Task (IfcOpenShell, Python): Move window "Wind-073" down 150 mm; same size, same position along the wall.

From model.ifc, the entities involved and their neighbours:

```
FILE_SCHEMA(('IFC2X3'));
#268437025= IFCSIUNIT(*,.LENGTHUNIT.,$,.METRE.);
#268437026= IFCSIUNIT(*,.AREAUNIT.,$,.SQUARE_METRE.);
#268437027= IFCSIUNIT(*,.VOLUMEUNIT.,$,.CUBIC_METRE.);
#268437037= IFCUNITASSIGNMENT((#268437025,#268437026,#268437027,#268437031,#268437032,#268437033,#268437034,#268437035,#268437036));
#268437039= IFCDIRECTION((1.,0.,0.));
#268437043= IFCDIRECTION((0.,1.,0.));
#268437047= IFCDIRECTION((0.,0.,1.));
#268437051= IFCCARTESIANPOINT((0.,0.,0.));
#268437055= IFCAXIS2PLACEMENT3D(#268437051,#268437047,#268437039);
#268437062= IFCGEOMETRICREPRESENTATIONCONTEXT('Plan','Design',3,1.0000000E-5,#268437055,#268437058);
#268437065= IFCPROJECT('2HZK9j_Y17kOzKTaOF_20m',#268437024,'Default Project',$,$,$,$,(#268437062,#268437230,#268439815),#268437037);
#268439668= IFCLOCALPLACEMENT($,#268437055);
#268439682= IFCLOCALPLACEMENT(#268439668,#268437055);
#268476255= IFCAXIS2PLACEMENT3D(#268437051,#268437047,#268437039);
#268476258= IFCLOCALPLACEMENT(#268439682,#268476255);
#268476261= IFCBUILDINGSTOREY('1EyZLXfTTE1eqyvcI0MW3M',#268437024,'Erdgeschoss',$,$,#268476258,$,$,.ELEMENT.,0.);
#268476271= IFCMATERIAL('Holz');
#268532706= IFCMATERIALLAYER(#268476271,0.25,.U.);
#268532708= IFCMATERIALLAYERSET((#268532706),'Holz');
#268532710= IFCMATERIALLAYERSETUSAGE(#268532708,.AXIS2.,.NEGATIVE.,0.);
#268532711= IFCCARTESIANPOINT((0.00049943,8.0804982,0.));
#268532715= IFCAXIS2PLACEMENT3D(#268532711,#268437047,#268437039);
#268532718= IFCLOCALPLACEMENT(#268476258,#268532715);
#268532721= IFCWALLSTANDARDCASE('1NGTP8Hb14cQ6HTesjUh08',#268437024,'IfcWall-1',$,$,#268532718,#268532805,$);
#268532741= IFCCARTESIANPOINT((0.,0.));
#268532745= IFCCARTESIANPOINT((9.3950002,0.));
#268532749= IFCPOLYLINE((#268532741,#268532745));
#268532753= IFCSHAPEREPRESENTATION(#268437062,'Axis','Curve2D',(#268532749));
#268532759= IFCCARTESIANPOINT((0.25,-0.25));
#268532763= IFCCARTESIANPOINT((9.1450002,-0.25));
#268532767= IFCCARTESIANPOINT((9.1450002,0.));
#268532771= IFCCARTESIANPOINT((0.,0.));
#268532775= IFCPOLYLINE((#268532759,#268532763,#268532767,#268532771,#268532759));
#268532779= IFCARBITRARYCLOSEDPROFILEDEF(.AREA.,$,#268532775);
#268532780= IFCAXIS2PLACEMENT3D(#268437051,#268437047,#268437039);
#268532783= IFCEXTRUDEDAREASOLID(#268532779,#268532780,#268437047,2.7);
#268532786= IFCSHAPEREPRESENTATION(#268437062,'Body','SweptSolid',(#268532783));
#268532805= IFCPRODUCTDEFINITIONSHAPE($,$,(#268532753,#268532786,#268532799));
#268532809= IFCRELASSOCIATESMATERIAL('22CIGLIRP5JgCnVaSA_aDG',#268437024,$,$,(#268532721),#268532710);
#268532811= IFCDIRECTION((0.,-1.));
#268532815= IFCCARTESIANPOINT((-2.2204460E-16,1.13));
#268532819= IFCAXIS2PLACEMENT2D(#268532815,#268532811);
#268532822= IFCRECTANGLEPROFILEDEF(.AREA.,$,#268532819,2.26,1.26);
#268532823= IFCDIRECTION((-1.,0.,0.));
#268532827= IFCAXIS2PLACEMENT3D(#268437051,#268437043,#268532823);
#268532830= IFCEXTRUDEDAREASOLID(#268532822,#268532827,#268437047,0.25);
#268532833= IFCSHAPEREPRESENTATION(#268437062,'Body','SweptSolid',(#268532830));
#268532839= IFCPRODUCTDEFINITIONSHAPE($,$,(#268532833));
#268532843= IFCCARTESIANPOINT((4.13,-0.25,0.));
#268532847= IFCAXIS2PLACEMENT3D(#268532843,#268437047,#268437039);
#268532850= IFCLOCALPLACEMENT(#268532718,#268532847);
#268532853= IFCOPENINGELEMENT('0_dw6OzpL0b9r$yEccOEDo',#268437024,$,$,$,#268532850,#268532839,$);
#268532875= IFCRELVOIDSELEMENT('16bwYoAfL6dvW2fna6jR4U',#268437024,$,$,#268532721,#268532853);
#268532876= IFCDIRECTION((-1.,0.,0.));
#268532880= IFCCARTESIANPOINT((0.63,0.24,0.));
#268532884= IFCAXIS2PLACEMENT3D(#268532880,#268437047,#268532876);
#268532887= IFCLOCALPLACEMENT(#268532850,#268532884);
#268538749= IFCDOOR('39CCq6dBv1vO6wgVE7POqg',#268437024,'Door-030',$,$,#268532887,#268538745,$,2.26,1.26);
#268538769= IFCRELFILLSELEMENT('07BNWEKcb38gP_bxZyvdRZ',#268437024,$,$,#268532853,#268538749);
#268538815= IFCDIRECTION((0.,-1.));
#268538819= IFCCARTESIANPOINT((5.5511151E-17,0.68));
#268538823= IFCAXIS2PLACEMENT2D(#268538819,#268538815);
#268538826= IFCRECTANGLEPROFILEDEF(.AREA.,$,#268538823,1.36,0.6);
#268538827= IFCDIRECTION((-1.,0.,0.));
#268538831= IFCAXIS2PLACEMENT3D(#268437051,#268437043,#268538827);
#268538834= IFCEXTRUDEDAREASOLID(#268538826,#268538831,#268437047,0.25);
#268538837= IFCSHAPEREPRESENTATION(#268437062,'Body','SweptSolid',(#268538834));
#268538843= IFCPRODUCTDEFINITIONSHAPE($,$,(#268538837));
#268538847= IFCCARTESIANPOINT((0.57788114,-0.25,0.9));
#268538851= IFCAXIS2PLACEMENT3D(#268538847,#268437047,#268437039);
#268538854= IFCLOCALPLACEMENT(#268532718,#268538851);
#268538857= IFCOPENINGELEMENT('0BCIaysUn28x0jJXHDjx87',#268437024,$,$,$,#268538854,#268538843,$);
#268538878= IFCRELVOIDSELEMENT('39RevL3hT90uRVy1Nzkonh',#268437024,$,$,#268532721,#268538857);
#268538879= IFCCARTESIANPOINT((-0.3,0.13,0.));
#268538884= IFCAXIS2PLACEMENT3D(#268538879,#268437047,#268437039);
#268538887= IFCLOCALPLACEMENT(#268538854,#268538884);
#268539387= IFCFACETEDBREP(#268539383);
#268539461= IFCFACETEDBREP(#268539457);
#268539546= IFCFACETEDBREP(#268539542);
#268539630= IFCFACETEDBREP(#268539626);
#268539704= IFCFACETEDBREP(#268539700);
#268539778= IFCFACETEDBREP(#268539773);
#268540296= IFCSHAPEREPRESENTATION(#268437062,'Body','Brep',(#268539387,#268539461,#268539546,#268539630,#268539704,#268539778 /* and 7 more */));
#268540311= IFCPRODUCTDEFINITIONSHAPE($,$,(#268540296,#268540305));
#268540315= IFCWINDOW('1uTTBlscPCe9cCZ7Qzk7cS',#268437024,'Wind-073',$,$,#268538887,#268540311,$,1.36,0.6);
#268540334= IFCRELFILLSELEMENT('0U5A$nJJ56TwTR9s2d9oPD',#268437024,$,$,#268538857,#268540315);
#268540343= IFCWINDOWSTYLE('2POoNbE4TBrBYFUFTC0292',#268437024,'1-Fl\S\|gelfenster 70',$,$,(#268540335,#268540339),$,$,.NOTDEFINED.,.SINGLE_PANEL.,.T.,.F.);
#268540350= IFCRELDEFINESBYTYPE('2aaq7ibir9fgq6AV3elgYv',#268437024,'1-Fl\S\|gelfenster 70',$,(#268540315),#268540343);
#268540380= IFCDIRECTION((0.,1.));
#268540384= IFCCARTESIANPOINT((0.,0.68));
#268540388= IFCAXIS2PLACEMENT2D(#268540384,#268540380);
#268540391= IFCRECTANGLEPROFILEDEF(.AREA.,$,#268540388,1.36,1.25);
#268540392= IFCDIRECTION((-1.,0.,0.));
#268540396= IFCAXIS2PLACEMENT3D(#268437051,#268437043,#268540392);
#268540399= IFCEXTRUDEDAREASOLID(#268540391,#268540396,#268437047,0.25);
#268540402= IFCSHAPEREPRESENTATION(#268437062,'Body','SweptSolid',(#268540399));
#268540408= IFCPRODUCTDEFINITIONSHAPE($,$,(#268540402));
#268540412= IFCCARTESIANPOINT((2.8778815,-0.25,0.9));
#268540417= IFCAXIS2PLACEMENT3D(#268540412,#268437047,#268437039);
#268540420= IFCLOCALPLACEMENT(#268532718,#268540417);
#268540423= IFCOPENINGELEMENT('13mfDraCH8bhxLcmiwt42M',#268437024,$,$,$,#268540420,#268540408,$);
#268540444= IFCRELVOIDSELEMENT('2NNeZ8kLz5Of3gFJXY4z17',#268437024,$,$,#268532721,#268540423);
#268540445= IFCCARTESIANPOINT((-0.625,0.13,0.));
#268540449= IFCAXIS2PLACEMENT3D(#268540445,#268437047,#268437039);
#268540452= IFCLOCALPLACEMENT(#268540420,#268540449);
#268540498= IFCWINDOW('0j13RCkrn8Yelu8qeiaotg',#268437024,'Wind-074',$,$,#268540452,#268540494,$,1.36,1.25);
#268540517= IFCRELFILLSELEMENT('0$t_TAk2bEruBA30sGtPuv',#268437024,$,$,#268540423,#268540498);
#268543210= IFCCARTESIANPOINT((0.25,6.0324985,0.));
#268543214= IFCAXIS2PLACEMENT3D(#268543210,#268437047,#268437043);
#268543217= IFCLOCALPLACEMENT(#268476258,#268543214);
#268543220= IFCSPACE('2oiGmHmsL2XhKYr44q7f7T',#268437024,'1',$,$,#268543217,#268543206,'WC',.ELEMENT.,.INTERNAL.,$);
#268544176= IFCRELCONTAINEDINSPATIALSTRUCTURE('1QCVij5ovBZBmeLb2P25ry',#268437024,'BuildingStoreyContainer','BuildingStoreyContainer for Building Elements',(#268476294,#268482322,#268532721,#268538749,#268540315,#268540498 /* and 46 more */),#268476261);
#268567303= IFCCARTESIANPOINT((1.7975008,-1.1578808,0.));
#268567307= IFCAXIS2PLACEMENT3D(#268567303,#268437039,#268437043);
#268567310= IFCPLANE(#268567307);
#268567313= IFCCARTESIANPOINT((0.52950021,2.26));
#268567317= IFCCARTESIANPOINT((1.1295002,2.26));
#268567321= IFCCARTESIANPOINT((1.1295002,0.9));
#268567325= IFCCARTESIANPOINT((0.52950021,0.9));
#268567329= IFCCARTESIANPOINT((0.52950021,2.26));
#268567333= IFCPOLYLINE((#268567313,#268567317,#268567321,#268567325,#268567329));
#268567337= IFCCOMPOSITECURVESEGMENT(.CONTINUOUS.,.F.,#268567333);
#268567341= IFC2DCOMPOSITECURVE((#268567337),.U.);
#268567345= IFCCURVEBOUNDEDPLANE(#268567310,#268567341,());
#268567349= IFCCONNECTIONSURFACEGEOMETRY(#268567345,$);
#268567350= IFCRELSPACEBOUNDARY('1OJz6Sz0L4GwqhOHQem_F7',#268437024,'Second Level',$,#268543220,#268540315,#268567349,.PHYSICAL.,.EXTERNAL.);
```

```python
import numpy as np
import ifcopenshell
import ifcopenshell.api.geometry
import ifcopenshell.util.placement
import ifcopenshell.util.unit

model = ifcopenshell.open("model.ifc")
unit_scale = ifcopenshell.util.unit.calculate_unit_scale(model)

window = model.by_id(268540315)
opening = window.FillsVoids[0].RelatingOpeningElement
dz = -0.15

shift = np.array([0.0, 0.0, dz])
# The window is placed relative to its opening, so it follows when the opening moves.
matrix = ifcopenshell.util.placement.get_local_placement(opening.ObjectPlacement)
matrix[:3, 3] += shift
ifcopenshell.api.geometry.edit_object_placement(
    model, product=opening, matrix=matrix, is_si=False, should_transform_children=True
)

# Space boundary surfaces are stored in each space's coordinates; move them too.
for rel in window.ProvidesBoundaries:
    if not rel.ConnectionGeometry:
        continue
    surface = rel.ConnectionGeometry.SurfaceOnRelatingElement.BasisSurface
    space_matrix = ifcopenshell.util.placement.get_local_placement(rel.RelatingSpace.ObjectPlacement)
    point = np.array(surface.Position.Location.Coordinates) + space_matrix[:3, :3].T @ shift
    surface.Position = model.createIfcAxis2Placement3D(
        model.createIfcCartesianPoint(point.tolist()), surface.Position.Axis, surface.Position.RefDirection
    )

print(f"moved by {dz * unit_scale:+.3f} m")

model.write("model-out.ifc")
```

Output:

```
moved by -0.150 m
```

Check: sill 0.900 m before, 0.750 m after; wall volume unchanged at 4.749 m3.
